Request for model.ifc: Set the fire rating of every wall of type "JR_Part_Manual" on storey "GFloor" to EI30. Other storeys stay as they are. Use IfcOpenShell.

First a look at what the model holds.

```python
import ifcopenshell
import ifcopenshell.util.element

model = ifcopenshell.open("model.ifc")
print(model.schema)
storey = next(s for s in model.by_type("IfcBuildingStorey") if s.Name == "GFloor")
walls = [e for e in ifcopenshell.util.element.get_decomposition(storey) if e.is_a("IfcWall")]
seen = {}
for e in walls:
    element_type = ifcopenshell.util.element.get_type(e)
    key = (element_type.Name if element_type != e and element_type else None, ifcopenshell.util.element.get_pset(e, "Pset_WallCommon", "FireRating"))
    seen[key] = seen.get(key, 0) + 1
for (name, value), count in sorted(seen.items(), key=str):
    print(count, "x", name, "|", value)
```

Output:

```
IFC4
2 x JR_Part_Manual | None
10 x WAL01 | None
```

```python
import ifcopenshell
import ifcopenshell.api.pset
import ifcopenshell.util.element

model = ifcopenshell.open("model.ifc")

storey = next(s for s in model.by_type("IfcBuildingStorey") if s.Name == "GFloor")
walls = [e for e in ifcopenshell.util.element.get_decomposition(storey) if e.is_a("IfcWall")]

count = 0
for e in walls:
    element_type = ifcopenshell.util.element.get_type(e)
    if element_type in (None, e) or element_type.Name != "JR_Part_Manual":
        continue
    # add_pset returns the element's existing set when there is one.
    pset = ifcopenshell.api.pset.add_pset(model, product=e, name="Pset_WallCommon")
    ifcopenshell.api.pset.edit_pset(model, pset=pset, properties={"FireRating": "EI30"})
    count += 1

print(count, "walls updated")

model.write("model_rev.ifc")
```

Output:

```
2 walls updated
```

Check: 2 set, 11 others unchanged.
